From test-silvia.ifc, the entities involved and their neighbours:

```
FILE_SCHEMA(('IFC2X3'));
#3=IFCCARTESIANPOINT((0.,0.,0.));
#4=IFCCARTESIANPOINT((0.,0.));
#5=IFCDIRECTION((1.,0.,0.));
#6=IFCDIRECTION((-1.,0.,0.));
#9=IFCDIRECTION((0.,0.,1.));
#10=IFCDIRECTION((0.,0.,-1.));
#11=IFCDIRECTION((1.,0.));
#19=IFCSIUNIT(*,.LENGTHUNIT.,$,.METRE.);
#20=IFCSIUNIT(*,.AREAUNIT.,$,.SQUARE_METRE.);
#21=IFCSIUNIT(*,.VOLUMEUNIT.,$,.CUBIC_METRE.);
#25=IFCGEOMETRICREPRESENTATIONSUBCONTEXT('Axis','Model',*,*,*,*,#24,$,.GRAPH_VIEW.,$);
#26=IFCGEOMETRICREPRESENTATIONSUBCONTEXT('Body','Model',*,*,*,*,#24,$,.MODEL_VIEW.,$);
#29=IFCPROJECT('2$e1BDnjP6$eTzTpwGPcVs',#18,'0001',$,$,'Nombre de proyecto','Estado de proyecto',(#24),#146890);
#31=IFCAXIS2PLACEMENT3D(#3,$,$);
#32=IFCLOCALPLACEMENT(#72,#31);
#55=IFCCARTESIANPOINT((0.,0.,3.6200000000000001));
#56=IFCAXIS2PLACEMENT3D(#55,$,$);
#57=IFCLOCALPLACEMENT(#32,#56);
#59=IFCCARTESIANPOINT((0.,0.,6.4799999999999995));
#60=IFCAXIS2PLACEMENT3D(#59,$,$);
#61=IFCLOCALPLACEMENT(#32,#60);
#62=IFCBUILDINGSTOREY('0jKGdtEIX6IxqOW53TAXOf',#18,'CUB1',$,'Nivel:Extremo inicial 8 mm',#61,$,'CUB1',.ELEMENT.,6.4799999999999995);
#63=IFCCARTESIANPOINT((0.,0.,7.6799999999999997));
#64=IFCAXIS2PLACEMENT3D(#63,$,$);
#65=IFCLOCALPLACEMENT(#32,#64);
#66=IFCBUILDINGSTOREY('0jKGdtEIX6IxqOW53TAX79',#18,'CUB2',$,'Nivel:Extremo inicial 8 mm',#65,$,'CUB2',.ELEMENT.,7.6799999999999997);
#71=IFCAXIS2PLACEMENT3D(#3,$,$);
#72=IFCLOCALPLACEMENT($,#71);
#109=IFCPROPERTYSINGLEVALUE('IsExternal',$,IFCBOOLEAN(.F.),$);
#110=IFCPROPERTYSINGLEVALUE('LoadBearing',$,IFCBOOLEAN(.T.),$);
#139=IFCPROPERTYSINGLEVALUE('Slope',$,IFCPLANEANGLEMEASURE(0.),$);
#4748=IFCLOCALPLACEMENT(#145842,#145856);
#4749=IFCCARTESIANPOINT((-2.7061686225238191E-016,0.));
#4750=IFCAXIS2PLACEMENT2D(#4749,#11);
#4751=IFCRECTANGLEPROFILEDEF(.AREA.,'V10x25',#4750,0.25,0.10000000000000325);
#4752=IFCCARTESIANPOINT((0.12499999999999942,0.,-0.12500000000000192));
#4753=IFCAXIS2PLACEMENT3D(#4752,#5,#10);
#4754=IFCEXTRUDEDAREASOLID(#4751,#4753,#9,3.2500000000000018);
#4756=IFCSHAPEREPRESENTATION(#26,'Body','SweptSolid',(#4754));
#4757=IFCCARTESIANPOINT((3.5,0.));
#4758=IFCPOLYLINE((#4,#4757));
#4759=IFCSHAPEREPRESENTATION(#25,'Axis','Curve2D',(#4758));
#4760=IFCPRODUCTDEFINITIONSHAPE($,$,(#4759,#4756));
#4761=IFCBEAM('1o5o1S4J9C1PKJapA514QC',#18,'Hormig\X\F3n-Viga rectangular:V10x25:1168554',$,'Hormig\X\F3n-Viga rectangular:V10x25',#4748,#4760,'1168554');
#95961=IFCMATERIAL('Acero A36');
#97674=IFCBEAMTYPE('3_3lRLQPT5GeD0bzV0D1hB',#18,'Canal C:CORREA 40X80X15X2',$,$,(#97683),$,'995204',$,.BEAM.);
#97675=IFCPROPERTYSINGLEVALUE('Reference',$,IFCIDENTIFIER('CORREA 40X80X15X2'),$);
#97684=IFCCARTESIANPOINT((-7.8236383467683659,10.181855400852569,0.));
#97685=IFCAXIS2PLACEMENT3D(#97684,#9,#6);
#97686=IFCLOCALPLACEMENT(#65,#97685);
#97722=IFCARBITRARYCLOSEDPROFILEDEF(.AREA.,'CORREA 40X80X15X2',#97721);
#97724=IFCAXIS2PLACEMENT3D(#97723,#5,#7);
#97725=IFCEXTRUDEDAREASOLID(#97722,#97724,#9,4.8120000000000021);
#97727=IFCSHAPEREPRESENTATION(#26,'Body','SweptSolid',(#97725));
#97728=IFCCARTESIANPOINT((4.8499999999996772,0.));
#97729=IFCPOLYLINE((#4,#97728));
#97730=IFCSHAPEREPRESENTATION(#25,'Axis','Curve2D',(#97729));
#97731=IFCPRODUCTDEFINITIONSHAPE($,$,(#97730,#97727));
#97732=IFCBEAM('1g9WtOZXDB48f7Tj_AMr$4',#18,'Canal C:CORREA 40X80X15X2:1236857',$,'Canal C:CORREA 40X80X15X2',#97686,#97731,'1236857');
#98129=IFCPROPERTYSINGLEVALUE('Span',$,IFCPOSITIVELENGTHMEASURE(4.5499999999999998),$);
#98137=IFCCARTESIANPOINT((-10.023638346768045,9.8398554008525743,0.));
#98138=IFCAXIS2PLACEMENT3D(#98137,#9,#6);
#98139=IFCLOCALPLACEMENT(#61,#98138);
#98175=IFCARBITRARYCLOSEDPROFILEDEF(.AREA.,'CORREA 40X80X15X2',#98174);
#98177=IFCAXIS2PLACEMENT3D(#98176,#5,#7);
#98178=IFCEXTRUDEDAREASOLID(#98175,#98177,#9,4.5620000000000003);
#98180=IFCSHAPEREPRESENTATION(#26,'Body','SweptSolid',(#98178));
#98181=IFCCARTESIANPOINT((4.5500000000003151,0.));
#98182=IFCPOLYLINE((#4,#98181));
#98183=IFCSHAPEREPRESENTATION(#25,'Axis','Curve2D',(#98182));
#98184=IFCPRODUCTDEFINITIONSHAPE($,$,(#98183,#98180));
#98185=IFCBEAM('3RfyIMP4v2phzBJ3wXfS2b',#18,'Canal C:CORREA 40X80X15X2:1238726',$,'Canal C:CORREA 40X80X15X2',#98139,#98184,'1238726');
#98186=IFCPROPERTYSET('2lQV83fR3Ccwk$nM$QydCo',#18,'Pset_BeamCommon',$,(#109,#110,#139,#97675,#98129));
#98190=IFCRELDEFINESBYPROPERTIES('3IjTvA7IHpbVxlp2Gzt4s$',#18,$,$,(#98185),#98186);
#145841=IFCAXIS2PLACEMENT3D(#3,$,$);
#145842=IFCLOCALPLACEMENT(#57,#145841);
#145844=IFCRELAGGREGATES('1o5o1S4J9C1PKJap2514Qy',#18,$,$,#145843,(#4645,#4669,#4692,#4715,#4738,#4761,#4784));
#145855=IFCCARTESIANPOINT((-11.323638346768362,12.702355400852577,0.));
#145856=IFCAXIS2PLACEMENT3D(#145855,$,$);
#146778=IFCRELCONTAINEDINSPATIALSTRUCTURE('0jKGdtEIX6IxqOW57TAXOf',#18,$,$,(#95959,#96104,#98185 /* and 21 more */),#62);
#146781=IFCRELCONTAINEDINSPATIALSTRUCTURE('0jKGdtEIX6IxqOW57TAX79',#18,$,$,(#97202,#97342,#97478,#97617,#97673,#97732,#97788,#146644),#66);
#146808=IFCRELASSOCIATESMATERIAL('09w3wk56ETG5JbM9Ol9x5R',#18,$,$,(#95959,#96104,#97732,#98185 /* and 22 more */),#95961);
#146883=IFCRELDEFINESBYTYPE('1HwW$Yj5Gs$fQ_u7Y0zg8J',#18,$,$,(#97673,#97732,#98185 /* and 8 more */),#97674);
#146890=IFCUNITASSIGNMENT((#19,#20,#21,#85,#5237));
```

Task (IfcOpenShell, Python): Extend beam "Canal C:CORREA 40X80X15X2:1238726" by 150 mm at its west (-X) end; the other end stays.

```python
import numpy as np
import ifcopenshell
import ifcopenshell.api.pset
import ifcopenshell.util.element
import ifcopenshell.util.representation
import ifcopenshell.util.unit

model = ifcopenshell.open("test-silvia.ifc")
unit_scale = ifcopenshell.util.unit.calculate_unit_scale(model)

member = model.by_guid("3RfyIMP4v2phzBJ3wXfS2b")
change = 0.15 / unit_scale

# The extrusion runs towards the end named, so only its depth changes.
body = ifcopenshell.util.representation.get_representation(member, "Model", "Body")
solid = body.Items[0]
old_length = solid.Depth
solid.Depth += change

# Move the axis end point with it.
axis = next(r for r in member.Representation.Representations if r.RepresentationIdentifier == "Axis").Items[0]
start, end = (np.array(p.Coordinates) for p in axis.Points)
end = end + (end - start) / np.linalg.norm(end - start) * change
point = model.createIfcCartesianPoint(end.tolist())
axis.Points = [axis.Points[0], point]

# Update the stored length and volume.
pset = model.by_id(ifcopenshell.util.element.get_pset(member, "Pset_BeamCommon", should_inherit=False)["id"])
ifcopenshell.api.pset.edit_pset(model, pset=pset, properties={
    "Span": model.create_entity("IfcPositiveLengthMeasure", solid.Depth),
})

print(f"length {old_length:g} -> {solid.Depth:g}")

model.write("test-silvia_v2.ifc")
```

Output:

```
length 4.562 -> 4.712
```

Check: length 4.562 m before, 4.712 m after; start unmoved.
